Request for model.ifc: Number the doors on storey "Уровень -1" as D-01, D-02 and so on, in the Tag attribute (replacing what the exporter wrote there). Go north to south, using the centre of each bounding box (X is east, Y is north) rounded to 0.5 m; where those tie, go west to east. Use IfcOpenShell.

First a look at what the model holds.

```python
import ifcopenshell
import ifcopenshell.util.element
import ifcopenshell.util.placement

model = ifcopenshell.open("model.ifc")
print(model.schema)
storey = next(s for s in model.by_type("IfcBuildingStorey") if s.Name == "Уровень -1")
doors = [e for e in ifcopenshell.util.element.get_decomposition(storey) if e.is_a("IfcDoor")]
for e in sorted(doors, key=lambda e: e.id()):
    origin = ifcopenshell.util.placement.get_local_placement(e.ObjectPlacement)[:3, 3]
    print(e.id(), e.Tag, e.Name, origin.round(2) + 0.0, sep=" | ")
```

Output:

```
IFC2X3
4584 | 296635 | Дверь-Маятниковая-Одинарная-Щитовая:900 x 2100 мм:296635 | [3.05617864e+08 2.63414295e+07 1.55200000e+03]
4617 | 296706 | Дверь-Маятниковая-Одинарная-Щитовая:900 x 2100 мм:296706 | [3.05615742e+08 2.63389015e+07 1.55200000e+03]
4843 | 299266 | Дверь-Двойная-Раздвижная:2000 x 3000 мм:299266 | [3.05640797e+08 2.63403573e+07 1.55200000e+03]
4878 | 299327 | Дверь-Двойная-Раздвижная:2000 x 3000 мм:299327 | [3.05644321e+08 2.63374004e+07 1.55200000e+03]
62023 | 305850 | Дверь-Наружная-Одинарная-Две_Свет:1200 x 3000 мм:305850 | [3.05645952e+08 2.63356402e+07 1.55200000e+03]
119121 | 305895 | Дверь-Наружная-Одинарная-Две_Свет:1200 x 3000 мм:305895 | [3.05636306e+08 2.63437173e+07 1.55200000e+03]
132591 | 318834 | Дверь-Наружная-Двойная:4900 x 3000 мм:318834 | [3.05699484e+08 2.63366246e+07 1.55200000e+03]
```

```python
import ifcopenshell
import ifcopenshell.geom
import ifcopenshell.util.element
import ifcopenshell.util.shape

model = ifcopenshell.open("model.ifc")
settings = ifcopenshell.geom.settings()
settings.set("use-world-coords", True)


def centre(element):
    shape = ifcopenshell.geom.create_shape(settings, element)
    return ifcopenshell.util.shape.get_bbox_centroid(shape.geometry)


storey = next(s for s in model.by_type("IfcBuildingStorey") if s.Name == "Уровень -1")
doors = [e for e in ifcopenshell.util.element.get_decomposition(storey) if e.is_a("IfcDoor")]

# Insertion points can sit at a corner or the storey origin, so sort by the geometry (in metres).
centres = {e: centre(e) for e in doors}
doors.sort(key=lambda e: (-round(centres[e][1] / 0.5), centres[e][0]))

for i, e in enumerate(doors, start=1):
    number = f"D-{i:02d}"
    e.Tag = number
    print(e.id(), number)

model.write("model_v2.ifc")
```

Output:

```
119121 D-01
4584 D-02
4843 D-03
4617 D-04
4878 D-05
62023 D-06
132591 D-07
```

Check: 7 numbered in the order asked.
